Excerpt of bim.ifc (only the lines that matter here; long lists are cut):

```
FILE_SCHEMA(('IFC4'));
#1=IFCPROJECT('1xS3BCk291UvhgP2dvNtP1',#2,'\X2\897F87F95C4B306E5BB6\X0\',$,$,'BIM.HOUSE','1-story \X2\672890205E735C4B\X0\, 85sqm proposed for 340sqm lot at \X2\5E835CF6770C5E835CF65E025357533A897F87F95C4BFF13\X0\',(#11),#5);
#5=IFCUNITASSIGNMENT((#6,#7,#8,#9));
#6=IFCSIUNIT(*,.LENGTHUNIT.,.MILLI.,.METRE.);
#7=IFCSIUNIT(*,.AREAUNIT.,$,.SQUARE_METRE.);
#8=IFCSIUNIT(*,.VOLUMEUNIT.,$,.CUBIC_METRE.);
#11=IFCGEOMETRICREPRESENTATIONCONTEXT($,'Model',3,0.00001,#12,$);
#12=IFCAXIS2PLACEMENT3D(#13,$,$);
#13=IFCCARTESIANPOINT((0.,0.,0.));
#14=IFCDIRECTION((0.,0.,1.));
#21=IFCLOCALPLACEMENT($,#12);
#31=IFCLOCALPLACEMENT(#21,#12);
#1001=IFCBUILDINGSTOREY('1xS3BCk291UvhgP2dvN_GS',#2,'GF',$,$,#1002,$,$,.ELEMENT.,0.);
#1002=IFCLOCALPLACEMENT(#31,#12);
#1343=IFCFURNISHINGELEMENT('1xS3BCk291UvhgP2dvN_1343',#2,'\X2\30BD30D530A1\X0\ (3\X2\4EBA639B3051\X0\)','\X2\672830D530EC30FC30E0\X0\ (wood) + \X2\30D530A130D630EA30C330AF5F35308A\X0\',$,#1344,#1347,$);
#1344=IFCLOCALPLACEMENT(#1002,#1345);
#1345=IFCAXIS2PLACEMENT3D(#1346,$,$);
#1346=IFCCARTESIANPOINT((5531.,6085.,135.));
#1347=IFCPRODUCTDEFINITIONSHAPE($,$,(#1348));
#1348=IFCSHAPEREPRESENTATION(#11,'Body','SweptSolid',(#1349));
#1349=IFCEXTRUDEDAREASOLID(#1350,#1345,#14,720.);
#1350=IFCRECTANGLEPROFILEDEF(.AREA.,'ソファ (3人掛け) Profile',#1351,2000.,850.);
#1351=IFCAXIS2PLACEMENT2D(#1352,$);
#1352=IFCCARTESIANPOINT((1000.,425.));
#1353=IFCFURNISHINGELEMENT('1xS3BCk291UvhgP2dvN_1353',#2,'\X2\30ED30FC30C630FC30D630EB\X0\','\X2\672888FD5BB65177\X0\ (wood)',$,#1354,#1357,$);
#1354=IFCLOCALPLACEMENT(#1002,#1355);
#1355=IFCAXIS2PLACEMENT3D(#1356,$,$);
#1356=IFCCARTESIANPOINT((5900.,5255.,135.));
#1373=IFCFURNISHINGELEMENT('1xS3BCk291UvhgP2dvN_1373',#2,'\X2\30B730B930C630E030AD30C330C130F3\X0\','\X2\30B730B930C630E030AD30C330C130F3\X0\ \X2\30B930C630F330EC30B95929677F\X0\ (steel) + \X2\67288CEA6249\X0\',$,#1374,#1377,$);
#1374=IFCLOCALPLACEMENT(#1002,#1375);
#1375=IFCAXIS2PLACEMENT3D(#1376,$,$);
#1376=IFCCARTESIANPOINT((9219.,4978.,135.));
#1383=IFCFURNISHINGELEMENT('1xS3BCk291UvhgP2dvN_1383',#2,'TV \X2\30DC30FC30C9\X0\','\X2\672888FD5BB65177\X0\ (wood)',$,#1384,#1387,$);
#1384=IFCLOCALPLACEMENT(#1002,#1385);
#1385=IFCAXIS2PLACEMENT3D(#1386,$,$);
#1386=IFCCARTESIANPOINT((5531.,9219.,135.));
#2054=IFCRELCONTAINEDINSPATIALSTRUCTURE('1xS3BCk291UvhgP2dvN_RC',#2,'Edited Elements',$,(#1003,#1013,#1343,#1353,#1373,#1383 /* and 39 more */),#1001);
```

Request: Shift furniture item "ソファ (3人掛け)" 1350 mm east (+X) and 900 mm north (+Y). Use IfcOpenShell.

```python
import ifcopenshell
import ifcopenshell.api.geometry
import ifcopenshell.util.placement
import ifcopenshell.util.unit

model = ifcopenshell.open("bim.ifc")
unit_scale = ifcopenshell.util.unit.calculate_unit_scale(model)

item = model.by_guid("1xS3BCk291UvhgP2dvN_1343")
matrix = ifcopenshell.util.placement.get_local_placement(item.ObjectPlacement)
matrix[0, 3] += 1.35 / unit_scale
matrix[1, 3] += 0.9 / unit_scale
ifcopenshell.api.geometry.edit_object_placement(model, product=item, matrix=matrix, is_si=False)

print(ifcopenshell.util.placement.get_local_placement(item.ObjectPlacement).round(3) + 0.0)

model.write("bim_edited.ifc")
```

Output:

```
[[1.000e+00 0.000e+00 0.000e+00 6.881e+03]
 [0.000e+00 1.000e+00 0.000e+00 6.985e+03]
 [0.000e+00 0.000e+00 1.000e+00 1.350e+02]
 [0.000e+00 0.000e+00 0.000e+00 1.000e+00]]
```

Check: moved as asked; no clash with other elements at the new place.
